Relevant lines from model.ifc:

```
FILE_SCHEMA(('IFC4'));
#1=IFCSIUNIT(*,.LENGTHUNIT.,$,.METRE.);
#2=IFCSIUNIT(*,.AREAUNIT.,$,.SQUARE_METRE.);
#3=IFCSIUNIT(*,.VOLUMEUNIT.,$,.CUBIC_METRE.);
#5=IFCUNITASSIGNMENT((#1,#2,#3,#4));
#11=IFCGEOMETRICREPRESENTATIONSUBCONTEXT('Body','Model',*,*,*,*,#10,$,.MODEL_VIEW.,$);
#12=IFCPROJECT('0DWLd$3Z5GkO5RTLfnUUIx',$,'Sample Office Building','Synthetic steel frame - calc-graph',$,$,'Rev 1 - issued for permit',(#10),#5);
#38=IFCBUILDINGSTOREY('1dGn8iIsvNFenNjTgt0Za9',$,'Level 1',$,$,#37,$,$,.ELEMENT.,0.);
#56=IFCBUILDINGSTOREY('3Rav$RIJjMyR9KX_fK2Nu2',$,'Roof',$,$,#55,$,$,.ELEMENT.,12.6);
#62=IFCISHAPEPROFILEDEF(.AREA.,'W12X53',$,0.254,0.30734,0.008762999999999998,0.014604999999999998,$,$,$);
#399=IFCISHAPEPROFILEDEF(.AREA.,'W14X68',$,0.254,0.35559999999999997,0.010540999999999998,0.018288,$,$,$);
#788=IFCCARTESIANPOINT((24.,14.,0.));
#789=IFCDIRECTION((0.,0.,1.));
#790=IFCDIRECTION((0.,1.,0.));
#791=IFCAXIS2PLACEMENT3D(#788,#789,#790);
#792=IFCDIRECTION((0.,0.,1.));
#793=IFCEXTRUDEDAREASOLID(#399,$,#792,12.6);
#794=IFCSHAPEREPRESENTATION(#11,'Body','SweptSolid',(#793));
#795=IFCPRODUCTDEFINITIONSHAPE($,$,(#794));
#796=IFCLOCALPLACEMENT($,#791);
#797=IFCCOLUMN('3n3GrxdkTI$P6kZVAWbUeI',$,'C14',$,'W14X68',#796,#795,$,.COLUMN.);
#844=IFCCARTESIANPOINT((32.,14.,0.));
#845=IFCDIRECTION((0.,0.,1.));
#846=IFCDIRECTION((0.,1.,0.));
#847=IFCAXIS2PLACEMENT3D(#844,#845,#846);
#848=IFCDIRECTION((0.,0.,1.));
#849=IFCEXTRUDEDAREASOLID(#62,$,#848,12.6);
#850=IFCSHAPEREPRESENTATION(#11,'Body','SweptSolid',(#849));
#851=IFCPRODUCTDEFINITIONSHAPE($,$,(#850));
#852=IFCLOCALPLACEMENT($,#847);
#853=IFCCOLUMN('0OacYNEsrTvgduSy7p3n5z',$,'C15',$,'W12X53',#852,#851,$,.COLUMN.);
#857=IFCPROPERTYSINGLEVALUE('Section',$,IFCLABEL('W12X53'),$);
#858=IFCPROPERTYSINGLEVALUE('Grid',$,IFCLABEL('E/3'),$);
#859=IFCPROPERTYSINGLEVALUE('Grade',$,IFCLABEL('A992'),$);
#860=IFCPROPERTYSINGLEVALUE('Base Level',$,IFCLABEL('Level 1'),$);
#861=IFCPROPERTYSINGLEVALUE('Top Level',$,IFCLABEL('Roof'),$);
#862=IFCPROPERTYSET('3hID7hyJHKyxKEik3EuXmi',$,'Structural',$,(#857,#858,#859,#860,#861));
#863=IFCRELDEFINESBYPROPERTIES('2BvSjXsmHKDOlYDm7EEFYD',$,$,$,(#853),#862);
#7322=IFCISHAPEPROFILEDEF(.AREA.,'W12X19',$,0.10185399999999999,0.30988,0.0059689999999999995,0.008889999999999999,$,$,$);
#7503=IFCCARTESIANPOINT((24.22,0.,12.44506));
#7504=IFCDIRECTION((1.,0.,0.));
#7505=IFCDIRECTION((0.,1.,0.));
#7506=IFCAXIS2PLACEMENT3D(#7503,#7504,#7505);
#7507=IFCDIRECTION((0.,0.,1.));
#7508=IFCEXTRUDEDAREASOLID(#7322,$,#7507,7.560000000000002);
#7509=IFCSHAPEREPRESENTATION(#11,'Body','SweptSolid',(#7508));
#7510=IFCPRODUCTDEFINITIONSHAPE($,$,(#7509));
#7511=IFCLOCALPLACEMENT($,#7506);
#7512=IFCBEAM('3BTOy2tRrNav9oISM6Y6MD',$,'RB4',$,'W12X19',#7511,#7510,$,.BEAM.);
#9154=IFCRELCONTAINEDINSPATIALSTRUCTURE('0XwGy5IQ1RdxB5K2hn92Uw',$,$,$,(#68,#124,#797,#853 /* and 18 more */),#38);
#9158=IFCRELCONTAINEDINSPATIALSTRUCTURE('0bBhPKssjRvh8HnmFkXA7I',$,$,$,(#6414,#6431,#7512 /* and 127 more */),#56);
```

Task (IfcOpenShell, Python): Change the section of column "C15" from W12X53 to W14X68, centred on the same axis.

```python
import ifcopenshell
import ifcopenshell.api.pset
import ifcopenshell.util.element
import ifcopenshell.util.representation

model = ifcopenshell.open("model.ifc")

member = model.by_guid("0OacYNEsrTvgduSy7p3n5z")
source = next(p for p in model.by_type("IfcIShapeProfileDef") if p.ProfileName == "W14X68")

body = ifcopenshell.util.representation.get_representation(member, "Model", "Body")
solid = body.Items[0]
old_profile = solid.SweptArea

# Copy the section's sizes but keep this member's own profile position.
profile = ifcopenshell.util.element.copy(model, source)
profile.Position = old_profile.Position
solid.SweptArea = profile
if not model.get_total_inverses(old_profile):
    ifcopenshell.util.element.remove_deep2(model, old_profile)
member.ObjectType = member.ObjectType.replace("W12X53", "W14X68")
pset = model.by_id(ifcopenshell.util.element.get_pset(member, "Structural", should_inherit=False)["id"])
ifcopenshell.api.pset.edit_pset(model, pset=pset, properties={"Section": "W14X68"})

print(solid.SweptArea)

model.write("model_rev.ifc")
```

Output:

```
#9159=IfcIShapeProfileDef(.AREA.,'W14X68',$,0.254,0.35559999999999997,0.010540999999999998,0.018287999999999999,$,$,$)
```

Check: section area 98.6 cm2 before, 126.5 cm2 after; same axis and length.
